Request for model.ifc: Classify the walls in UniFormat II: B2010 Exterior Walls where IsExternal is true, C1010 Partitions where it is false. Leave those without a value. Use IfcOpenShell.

First a look at what the model holds.

```python
import ifcopenshell
import ifcopenshell.util.element

model = ifcopenshell.open("model.ifc")
print(model.schema)
print("classifications:", [c.Name for c in model.by_type("IfcClassification")])
values = [ifcopenshell.util.element.get_pset(e, "Pset_WallCommon", "IsExternal") for e in model.by_type("IfcWall")]
for value in (True, False, None):
    print("IsExternal", value, values.count(value))
```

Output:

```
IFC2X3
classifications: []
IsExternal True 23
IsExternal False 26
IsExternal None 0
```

```python
import ifcopenshell
import ifcopenshell.api.classification
import ifcopenshell.util.element

model = ifcopenshell.open("model.ifc")

# IFC2X3 requires Source and Edition and has no link from the project to the system.
system = model.create_entity("IfcClassification", Source="ASTM", Edition="E1557", Name="UniFormat II")

walls = model.by_type("IfcWall")
external = {e: ifcopenshell.util.element.get_pset(e, "Pset_WallCommon", "IsExternal") for e in walls}
for flag, code, name in ((True, "B2010", "Exterior Walls"), (False, "C1010", "Partitions")):
    products = [e for e in walls if external[e] is flag]
    ifcopenshell.api.classification.add_reference(
        model, products=products, classification=system, identification=code, name=name
    )
    print(code, len(products))

model.write("model_rev.ifc")
```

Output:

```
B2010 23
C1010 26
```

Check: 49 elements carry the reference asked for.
